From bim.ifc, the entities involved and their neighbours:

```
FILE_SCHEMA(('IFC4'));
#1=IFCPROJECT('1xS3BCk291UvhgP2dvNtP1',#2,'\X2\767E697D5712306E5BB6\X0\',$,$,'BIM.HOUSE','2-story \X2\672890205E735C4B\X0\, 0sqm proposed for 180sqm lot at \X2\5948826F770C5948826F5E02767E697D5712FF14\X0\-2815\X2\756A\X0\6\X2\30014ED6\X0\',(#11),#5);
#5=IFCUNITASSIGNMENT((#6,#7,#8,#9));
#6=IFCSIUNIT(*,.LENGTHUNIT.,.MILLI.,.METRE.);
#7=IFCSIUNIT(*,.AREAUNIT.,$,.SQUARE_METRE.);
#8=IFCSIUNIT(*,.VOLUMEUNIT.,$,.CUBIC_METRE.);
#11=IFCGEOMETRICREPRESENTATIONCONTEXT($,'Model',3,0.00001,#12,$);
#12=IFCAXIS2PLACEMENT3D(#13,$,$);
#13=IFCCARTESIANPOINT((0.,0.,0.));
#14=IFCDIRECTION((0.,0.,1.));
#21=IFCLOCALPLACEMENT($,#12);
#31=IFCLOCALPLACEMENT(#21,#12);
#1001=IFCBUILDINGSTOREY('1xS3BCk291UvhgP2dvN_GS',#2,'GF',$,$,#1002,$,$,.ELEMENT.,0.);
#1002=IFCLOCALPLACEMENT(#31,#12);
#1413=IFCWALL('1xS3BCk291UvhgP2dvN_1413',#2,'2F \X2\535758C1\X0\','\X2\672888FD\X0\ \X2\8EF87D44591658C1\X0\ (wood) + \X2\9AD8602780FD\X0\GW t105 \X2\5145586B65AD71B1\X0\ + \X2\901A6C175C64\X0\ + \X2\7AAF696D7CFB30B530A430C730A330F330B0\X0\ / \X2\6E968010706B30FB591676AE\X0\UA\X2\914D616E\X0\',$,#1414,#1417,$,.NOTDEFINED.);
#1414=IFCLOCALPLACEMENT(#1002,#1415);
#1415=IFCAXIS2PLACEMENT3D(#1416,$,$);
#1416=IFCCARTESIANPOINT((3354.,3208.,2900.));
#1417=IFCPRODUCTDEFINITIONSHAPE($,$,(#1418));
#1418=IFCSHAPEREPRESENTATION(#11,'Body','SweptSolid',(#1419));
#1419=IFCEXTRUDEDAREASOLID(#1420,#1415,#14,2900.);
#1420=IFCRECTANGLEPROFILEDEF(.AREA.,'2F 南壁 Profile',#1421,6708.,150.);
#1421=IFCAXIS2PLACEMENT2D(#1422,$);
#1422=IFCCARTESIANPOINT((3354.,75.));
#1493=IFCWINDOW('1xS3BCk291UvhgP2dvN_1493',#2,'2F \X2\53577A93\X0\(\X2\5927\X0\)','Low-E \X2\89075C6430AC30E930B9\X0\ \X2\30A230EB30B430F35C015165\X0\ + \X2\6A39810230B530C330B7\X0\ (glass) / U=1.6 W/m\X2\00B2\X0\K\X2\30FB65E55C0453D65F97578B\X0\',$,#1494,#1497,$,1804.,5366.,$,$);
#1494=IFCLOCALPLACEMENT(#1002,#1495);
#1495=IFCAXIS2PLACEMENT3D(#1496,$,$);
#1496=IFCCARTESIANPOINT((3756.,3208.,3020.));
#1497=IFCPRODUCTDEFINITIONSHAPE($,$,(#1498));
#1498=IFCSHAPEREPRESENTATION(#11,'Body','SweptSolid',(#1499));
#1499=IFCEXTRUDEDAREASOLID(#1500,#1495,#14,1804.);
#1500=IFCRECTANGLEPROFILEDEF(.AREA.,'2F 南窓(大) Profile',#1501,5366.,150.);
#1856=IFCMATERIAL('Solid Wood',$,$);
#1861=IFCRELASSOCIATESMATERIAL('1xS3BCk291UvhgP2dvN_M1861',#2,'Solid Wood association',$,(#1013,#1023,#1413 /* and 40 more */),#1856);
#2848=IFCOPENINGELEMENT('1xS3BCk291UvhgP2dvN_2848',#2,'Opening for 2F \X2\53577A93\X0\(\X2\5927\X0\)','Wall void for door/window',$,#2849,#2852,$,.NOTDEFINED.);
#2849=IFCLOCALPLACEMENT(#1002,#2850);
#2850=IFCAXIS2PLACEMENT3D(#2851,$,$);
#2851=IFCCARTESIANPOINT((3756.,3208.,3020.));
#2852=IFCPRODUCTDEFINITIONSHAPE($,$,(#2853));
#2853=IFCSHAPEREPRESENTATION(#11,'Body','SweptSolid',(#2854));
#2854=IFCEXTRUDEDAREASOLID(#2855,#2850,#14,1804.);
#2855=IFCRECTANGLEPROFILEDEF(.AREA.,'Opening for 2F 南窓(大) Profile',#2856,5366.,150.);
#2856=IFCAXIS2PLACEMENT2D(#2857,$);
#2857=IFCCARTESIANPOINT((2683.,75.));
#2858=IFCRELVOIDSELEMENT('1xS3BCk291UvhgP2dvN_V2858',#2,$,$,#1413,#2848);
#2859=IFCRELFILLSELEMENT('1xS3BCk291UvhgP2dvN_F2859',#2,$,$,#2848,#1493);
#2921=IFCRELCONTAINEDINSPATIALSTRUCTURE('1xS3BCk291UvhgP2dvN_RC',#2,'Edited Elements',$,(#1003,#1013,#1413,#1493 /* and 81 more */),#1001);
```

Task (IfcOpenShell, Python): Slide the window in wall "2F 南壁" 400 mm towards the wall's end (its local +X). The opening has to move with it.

```python
import ifcopenshell
import ifcopenshell.api.geometry
import ifcopenshell.util.placement
import ifcopenshell.util.unit

model = ifcopenshell.open("bim.ifc")
unit_scale = ifcopenshell.util.unit.calculate_unit_scale(model)

window = model.by_guid("1xS3BCk291UvhgP2dvN_1493")
opening = window.FillsVoids[0].RelatingOpeningElement
wall = opening.VoidsElements[0].RelatingBuildingElement

wall_matrix = ifcopenshell.util.placement.get_local_placement(wall.ObjectPlacement)
shift = wall_matrix[:3, 0] * 0.4 / unit_scale
before = ifcopenshell.util.placement.get_local_placement(window.ObjectPlacement)[:3, 3].copy()

# The window is not placed relative to its opening, so move both.
for product in (opening, window):
    matrix = ifcopenshell.util.placement.get_local_placement(product.ObjectPlacement)
    matrix[:3, 3] += shift
    ifcopenshell.api.geometry.edit_object_placement(model, product=product, matrix=matrix, is_si=False)

after = ifcopenshell.util.placement.get_local_placement(window.ObjectPlacement)[:3, 3]
print("window moved by", (after - before).round(3) + 0.0)

model.write("bim-out.ifc")
```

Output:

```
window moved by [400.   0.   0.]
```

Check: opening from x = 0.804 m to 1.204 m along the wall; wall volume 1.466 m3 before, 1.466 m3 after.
